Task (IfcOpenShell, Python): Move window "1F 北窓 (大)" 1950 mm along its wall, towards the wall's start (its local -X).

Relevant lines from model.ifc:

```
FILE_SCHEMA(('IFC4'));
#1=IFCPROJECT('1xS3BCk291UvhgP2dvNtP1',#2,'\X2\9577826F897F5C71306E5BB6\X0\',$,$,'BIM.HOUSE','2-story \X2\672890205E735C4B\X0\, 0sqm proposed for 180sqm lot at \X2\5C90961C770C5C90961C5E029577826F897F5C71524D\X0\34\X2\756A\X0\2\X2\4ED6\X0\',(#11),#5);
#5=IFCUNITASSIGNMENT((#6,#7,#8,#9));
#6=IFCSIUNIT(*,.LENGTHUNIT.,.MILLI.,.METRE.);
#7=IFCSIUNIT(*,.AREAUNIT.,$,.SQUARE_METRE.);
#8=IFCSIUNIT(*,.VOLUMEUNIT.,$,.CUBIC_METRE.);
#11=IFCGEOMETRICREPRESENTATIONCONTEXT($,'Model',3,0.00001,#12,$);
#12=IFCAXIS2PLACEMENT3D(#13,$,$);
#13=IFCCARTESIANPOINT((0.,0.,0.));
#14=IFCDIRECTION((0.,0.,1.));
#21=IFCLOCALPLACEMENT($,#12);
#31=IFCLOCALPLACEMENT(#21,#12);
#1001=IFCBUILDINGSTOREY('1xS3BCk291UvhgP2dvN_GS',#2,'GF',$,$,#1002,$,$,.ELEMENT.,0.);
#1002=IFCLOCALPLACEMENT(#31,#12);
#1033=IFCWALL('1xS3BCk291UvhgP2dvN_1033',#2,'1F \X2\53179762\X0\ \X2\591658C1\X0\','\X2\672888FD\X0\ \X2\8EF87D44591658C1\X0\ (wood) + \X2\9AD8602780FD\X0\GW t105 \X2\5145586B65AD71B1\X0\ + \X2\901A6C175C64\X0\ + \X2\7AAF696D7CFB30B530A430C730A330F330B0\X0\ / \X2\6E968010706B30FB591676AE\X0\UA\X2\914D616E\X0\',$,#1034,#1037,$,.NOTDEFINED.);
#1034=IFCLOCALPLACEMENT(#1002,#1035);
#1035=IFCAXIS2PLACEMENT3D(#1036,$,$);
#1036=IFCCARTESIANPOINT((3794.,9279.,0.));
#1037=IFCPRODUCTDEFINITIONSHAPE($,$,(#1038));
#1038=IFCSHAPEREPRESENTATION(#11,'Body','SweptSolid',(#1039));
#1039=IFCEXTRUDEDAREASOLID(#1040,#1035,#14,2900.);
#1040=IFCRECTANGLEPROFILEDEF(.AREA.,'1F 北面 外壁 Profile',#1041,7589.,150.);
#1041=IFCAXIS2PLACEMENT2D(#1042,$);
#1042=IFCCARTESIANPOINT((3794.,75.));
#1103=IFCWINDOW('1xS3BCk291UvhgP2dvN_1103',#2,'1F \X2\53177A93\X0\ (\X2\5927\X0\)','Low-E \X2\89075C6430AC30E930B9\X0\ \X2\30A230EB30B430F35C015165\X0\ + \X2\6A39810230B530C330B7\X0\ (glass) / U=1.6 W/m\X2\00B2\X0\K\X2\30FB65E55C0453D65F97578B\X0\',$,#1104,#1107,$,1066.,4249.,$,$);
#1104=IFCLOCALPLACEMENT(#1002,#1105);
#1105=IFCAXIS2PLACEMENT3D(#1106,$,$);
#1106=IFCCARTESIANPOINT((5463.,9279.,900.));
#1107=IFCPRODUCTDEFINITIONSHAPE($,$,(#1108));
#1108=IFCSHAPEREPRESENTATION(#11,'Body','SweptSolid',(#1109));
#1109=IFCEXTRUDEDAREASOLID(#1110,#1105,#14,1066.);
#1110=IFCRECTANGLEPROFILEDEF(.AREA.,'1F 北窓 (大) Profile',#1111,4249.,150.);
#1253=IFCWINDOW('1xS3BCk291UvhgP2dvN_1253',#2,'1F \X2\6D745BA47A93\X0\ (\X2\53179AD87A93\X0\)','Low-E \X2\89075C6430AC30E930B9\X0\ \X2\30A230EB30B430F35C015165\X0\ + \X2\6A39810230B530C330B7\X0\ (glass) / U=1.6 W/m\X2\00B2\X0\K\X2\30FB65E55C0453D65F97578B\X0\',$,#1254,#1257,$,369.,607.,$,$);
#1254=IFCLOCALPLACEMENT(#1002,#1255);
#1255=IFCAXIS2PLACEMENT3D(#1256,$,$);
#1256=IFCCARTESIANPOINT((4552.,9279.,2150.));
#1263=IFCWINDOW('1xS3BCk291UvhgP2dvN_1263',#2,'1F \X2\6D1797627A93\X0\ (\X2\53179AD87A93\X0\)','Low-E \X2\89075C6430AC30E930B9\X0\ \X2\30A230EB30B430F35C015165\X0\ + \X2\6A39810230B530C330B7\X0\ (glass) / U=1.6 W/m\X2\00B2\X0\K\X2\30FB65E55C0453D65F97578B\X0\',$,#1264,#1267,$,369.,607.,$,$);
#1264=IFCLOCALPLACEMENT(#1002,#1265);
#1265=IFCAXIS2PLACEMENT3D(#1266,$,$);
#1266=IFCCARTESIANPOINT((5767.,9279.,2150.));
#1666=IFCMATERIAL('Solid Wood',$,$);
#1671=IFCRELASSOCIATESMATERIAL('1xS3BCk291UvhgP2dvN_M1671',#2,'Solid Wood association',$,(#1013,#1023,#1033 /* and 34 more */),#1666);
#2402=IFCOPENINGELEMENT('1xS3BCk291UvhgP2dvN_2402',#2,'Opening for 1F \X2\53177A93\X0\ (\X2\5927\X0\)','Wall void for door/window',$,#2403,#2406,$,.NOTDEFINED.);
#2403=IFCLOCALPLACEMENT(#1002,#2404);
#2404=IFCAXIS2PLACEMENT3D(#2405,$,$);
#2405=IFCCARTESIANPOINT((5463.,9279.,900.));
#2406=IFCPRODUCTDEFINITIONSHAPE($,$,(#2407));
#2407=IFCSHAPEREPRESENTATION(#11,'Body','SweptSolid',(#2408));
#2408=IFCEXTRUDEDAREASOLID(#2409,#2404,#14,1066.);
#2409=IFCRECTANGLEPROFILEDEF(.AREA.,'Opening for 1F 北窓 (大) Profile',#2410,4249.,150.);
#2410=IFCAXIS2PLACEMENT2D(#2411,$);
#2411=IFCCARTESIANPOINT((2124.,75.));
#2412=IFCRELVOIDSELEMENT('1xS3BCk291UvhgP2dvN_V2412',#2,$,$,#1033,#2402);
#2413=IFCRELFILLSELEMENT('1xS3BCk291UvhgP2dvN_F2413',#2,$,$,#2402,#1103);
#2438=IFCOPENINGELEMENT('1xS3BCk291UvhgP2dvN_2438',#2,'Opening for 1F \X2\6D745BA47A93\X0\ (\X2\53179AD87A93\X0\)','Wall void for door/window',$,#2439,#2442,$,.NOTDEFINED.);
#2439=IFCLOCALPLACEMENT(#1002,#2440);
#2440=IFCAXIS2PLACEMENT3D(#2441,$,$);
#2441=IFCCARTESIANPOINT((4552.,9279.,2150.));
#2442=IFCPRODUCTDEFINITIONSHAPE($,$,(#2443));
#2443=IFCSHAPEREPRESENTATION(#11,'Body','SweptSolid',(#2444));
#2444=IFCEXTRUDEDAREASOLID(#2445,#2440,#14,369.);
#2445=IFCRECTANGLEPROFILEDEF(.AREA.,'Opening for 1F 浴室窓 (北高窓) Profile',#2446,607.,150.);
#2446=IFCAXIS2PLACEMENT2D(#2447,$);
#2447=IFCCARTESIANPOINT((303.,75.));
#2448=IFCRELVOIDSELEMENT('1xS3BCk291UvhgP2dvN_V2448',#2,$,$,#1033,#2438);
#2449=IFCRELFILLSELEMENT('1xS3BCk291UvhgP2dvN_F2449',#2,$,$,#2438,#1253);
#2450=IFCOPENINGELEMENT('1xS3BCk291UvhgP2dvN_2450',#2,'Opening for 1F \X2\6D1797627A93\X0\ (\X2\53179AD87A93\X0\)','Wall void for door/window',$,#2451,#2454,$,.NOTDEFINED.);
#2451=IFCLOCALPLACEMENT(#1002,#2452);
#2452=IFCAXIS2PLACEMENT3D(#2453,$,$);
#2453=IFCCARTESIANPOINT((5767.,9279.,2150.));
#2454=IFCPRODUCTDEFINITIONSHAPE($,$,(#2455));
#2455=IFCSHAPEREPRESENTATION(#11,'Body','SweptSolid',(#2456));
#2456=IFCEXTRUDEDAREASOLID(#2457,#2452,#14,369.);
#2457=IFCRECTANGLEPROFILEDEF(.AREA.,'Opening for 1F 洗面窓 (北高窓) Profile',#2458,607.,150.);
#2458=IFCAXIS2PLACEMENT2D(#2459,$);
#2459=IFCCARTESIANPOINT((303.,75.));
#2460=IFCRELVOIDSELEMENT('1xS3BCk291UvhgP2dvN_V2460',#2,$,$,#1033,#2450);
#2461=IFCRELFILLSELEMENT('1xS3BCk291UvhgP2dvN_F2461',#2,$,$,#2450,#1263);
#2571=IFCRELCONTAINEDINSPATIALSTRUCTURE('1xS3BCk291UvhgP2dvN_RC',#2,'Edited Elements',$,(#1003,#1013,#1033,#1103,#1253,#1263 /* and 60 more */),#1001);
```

```python
import ifcopenshell
import ifcopenshell.api.geometry
import ifcopenshell.util.placement
import ifcopenshell.util.unit

model = ifcopenshell.open("model.ifc")
unit_scale = ifcopenshell.util.unit.calculate_unit_scale(model)

window = model.by_id(1103)
opening = window.FillsVoids[0].RelatingOpeningElement
wall = opening.VoidsElements[0].RelatingBuildingElement

wall_matrix = ifcopenshell.util.placement.get_local_placement(wall.ObjectPlacement)
shift = wall_matrix[:3, 0] * -1.95 / unit_scale
before = ifcopenshell.util.placement.get_local_placement(window.ObjectPlacement)[:3, 3].copy()

# The window is not placed relative to its opening, so move both.
for product in (opening, window):
    matrix = ifcopenshell.util.placement.get_local_placement(product.ObjectPlacement)
    matrix[:3, 3] += shift
    ifcopenshell.api.geometry.edit_object_placement(model, product=product, matrix=matrix, is_si=False)

after = ifcopenshell.util.placement.get_local_placement(window.ObjectPlacement)[:3, 3]
print("window moved by", (after - before).round(3) + 0.0)

model.write("model_rev.ifc")
```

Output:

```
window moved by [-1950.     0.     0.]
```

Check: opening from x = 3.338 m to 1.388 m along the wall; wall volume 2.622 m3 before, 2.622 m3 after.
